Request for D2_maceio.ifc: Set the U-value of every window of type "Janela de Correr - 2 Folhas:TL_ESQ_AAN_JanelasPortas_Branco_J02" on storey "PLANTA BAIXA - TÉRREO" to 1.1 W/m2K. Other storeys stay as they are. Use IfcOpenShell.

First a look at what the model holds.

```python
import ifcopenshell
import ifcopenshell.util.element

model = ifcopenshell.open("D2_maceio.ifc")
print(model.schema)
storey = next(s for s in model.by_type("IfcBuildingStorey") if s.Name == "PLANTA BAIXA - TÉRREO")
windows = [e for e in ifcopenshell.util.element.get_decomposition(storey) if e.is_a("IfcWindow")]
seen = {}
for e in windows:
    element_type = ifcopenshell.util.element.get_type(e)
    key = (element_type.Name if element_type != e and element_type else None, ifcopenshell.util.element.get_pset(e, "Pset_WindowCommon", "ThermalTransmittance"))
    seen[key] = seen.get(key, 0) + 1
for (name, value), count in sorted(seen.items(), key=str):
    print(count, "x", name, "|", value)
```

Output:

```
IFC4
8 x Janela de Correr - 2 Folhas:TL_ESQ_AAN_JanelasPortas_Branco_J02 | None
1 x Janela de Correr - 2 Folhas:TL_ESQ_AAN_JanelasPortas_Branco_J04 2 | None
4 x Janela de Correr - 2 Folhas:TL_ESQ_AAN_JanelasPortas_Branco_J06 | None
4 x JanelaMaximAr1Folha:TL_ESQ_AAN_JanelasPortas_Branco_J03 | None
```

```python
import ifcopenshell
import ifcopenshell.api.pset
import ifcopenshell.util.element

model = ifcopenshell.open("D2_maceio.ifc")

storey = next(s for s in model.by_type("IfcBuildingStorey") if s.Name == "PLANTA BAIXA - TÉRREO")
windows = [e for e in ifcopenshell.util.element.get_decomposition(storey) if e.is_a("IfcWindow")]

count = 0
for e in windows:
    element_type = ifcopenshell.util.element.get_type(e)
    if element_type in (None, e) or element_type.Name != "Janela de Correr - 2 Folhas:TL_ESQ_AAN_JanelasPortas_Branco_J02":
        continue
    # add_pset returns the element's existing set when there is one.
    pset = ifcopenshell.api.pset.add_pset(model, product=e, name="Pset_WindowCommon")
    ifcopenshell.api.pset.edit_pset(model, pset=pset, properties={"ThermalTransmittance": 1.1})
    count += 1

print(count, "windows updated")

model.write("D2_maceio_v2.ifc")
```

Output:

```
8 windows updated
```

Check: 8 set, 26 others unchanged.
